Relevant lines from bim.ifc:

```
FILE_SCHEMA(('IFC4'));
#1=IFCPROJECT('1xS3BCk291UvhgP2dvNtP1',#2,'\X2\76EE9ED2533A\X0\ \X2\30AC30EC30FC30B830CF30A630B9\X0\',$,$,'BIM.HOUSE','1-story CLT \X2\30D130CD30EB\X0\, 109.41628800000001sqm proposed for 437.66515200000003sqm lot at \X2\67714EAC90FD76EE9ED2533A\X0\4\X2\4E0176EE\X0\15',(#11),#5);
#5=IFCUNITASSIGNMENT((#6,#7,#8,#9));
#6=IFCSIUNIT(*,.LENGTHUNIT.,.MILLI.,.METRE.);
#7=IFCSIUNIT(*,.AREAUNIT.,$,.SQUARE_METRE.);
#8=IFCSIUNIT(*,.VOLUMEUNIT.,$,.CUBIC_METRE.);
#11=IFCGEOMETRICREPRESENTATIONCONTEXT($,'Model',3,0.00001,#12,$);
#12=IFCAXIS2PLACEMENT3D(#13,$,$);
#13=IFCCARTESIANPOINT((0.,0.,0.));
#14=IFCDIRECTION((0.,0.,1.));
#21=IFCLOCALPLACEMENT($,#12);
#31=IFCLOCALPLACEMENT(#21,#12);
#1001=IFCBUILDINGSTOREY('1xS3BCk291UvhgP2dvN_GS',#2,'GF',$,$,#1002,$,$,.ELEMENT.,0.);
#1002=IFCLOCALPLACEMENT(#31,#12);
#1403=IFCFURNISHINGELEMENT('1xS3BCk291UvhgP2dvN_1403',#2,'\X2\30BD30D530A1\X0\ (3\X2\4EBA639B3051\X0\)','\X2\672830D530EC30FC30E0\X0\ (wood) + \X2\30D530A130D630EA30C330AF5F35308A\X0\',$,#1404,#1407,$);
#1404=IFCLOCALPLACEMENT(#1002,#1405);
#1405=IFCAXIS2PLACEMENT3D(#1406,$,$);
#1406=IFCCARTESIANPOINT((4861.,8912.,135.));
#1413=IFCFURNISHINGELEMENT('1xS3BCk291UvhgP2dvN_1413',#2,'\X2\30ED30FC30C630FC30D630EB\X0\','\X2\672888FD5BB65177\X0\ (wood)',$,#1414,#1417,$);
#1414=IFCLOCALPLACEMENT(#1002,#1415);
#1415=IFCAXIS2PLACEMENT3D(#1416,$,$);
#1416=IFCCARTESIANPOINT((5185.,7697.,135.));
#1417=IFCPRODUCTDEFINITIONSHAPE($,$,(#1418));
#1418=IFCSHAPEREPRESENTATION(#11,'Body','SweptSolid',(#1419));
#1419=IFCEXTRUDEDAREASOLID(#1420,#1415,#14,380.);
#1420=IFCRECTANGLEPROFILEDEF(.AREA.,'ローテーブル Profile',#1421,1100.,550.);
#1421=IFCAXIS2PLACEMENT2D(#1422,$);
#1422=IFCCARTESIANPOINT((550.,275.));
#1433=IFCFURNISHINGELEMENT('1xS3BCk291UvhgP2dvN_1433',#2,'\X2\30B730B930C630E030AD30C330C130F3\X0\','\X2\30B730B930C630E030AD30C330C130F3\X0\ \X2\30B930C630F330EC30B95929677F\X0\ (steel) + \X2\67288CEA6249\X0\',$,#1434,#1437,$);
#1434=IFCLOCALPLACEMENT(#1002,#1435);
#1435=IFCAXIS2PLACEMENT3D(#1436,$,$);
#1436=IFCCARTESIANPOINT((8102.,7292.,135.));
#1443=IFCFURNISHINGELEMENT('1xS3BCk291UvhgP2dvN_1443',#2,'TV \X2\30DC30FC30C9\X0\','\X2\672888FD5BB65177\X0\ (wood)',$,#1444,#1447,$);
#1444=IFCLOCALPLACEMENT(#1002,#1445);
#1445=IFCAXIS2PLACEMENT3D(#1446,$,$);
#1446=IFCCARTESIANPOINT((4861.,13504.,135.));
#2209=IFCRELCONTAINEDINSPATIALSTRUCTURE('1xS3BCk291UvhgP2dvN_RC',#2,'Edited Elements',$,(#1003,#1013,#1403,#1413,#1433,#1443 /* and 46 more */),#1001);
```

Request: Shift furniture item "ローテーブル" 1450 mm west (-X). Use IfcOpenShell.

```python
import ifcopenshell
import ifcopenshell.api.geometry
import ifcopenshell.util.placement

model = ifcopenshell.open("bim.ifc")

item = model.by_guid("1xS3BCk291UvhgP2dvN_1413")
matrix = ifcopenshell.util.placement.get_local_placement(item.ObjectPlacement)
matrix[0, 3] -= 1450.0
ifcopenshell.api.geometry.edit_object_placement(model, product=item, matrix=matrix, is_si=False)

print(ifcopenshell.util.placement.get_local_placement(item.ObjectPlacement).round(3) + 0.0)

model.write("bim_rev.ifc")
```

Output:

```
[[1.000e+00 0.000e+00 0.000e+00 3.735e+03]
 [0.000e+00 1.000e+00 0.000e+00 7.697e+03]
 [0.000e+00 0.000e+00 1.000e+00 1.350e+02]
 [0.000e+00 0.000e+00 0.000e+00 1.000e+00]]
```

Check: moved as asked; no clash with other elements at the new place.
